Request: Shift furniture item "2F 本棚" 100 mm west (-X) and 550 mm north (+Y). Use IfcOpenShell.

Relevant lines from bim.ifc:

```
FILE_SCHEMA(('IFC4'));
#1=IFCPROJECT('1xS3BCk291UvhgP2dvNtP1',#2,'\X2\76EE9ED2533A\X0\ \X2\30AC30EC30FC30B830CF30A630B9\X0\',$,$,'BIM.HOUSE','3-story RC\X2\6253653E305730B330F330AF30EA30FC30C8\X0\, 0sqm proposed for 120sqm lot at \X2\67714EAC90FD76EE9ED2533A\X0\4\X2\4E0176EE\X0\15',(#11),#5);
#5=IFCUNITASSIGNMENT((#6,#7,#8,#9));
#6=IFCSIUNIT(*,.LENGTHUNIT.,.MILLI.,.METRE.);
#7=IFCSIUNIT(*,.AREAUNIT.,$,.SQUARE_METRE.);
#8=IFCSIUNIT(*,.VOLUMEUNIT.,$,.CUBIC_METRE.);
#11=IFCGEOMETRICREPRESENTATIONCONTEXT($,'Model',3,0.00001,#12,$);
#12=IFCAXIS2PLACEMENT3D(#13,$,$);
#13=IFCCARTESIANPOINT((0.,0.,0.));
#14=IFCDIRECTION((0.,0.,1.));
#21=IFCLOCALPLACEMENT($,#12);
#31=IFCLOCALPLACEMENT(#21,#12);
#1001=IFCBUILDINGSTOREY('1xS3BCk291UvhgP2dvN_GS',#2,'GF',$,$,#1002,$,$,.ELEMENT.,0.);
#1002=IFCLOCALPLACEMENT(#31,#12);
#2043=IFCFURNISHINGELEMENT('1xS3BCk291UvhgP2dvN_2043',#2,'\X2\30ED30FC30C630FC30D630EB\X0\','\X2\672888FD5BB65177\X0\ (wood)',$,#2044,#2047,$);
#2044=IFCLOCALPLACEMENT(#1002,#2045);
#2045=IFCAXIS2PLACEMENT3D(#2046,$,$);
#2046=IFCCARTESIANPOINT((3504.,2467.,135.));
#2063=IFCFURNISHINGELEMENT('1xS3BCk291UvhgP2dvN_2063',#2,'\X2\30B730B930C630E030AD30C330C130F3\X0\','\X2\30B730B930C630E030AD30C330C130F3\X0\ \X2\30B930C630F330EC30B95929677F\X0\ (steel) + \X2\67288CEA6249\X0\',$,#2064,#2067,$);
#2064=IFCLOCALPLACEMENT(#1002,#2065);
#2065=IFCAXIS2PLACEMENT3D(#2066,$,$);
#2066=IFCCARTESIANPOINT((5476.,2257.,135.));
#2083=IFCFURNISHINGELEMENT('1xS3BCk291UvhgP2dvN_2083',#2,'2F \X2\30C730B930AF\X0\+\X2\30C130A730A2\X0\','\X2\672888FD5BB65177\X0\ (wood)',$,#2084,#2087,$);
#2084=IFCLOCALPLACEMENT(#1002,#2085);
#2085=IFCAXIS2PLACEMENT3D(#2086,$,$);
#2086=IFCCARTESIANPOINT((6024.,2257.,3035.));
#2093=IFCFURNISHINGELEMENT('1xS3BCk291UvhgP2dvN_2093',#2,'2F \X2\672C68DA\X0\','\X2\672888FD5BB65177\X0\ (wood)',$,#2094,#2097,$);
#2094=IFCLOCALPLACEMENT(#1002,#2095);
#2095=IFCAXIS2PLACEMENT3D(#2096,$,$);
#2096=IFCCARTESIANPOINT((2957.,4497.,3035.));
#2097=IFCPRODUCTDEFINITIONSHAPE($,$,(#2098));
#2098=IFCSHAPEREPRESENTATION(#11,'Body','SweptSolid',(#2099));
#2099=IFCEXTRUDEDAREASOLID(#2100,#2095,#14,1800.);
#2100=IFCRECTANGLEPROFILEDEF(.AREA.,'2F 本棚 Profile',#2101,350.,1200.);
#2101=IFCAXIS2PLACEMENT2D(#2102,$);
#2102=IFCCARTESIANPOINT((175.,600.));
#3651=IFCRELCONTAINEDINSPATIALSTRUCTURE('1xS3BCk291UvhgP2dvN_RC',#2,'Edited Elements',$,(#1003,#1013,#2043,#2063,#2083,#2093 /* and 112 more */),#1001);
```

```python
import ifcopenshell
import ifcopenshell.api.geometry
import ifcopenshell.util.placement
import ifcopenshell.util.unit

model = ifcopenshell.open("bim.ifc")
unit_scale = ifcopenshell.util.unit.calculate_unit_scale(model)

item = model.by_guid("1xS3BCk291UvhgP2dvN_2093")
matrix = ifcopenshell.util.placement.get_local_placement(item.ObjectPlacement)
matrix[0, 3] -= 0.1 / unit_scale
matrix[1, 3] += 0.55 / unit_scale
ifcopenshell.api.geometry.edit_object_placement(model, product=item, matrix=matrix, is_si=False)

print(ifcopenshell.util.placement.get_local_placement(item.ObjectPlacement).round(3) + 0.0)

model.write("bim-out.ifc")
```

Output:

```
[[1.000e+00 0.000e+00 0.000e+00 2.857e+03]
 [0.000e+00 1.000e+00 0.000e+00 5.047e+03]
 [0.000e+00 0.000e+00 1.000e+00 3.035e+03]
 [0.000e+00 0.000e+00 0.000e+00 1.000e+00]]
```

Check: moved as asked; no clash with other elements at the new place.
